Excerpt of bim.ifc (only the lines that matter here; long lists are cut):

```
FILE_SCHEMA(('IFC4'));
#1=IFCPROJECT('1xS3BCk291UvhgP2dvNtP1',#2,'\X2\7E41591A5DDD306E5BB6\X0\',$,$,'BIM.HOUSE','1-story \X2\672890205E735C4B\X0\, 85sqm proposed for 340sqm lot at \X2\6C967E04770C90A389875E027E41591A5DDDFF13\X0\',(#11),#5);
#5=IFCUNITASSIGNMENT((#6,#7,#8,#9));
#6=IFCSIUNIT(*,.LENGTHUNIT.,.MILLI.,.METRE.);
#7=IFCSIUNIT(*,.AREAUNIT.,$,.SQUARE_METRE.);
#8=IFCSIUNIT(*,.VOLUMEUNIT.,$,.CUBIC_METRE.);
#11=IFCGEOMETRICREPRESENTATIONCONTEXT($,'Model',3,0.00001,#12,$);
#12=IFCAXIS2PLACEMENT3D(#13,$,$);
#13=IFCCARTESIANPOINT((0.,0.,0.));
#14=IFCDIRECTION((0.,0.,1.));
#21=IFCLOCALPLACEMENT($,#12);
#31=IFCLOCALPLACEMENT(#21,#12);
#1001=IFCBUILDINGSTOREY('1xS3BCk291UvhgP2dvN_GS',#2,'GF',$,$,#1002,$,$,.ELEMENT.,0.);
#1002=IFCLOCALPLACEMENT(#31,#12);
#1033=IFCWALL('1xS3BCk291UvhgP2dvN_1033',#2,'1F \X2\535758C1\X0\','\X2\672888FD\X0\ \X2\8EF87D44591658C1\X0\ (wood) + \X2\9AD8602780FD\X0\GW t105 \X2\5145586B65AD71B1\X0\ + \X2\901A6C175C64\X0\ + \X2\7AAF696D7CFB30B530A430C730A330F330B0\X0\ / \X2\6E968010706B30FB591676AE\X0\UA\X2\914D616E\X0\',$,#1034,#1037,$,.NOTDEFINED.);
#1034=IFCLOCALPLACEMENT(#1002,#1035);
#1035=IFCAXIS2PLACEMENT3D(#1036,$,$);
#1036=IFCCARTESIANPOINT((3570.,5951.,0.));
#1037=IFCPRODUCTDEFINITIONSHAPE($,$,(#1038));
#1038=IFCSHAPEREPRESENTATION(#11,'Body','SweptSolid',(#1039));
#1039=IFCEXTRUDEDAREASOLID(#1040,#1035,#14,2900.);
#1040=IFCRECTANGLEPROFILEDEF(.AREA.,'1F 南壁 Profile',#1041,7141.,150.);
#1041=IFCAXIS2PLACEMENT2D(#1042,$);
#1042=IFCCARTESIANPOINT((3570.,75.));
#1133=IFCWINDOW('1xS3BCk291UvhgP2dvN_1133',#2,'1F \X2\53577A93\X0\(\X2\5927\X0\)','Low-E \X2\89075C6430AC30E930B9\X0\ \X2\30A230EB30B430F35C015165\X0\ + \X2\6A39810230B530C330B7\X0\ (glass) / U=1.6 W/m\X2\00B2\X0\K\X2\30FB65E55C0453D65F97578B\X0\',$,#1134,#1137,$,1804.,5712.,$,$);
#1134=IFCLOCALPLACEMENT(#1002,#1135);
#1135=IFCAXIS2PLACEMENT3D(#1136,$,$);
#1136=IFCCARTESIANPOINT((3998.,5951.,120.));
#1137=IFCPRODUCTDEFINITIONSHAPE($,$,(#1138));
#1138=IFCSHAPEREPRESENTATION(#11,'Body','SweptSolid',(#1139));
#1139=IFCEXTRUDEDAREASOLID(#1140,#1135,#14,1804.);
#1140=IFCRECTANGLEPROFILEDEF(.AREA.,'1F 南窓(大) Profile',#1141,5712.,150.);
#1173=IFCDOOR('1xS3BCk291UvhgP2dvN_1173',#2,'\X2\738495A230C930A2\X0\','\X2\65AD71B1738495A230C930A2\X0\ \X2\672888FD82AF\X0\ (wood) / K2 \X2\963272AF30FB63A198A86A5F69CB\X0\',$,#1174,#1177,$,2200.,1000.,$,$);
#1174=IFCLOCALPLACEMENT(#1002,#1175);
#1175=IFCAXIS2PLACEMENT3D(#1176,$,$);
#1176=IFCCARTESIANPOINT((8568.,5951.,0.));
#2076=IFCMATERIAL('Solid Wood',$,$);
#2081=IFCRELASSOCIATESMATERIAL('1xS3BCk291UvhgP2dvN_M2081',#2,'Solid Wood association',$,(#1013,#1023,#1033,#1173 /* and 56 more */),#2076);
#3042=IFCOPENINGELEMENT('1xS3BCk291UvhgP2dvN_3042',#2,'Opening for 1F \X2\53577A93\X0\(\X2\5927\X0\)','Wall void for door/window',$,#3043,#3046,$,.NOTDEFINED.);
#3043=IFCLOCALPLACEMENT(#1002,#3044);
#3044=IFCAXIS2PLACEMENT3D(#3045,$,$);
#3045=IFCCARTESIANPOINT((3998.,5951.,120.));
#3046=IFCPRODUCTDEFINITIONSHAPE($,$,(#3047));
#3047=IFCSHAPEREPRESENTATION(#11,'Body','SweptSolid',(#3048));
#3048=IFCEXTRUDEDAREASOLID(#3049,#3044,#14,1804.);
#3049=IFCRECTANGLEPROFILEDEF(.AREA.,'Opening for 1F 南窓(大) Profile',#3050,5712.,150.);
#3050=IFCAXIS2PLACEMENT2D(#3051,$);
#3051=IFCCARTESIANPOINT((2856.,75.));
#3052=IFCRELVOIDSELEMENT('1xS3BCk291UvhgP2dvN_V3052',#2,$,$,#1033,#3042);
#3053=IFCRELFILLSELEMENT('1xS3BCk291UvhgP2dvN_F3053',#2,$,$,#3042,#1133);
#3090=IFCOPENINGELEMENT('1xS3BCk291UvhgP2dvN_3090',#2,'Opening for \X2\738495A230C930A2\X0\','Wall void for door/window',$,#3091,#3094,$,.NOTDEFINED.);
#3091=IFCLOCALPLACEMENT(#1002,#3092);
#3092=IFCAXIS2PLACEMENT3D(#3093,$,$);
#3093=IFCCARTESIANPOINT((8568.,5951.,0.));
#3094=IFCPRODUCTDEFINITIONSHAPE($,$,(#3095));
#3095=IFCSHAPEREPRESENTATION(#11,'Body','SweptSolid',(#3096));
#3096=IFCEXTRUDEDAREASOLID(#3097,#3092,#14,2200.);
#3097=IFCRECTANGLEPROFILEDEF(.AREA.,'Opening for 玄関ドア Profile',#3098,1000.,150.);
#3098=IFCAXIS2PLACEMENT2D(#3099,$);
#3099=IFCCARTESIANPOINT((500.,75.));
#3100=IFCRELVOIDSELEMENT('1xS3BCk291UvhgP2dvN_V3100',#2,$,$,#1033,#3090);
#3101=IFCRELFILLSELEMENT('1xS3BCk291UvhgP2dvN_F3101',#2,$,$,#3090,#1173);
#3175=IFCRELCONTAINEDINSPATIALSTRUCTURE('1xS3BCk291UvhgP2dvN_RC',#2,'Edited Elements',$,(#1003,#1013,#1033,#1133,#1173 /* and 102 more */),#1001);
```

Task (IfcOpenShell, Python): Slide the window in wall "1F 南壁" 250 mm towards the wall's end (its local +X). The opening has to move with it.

```python
import ifcopenshell
import ifcopenshell.api.geometry
import ifcopenshell.util.placement
import ifcopenshell.util.unit

model = ifcopenshell.open("bim.ifc")
unit_scale = ifcopenshell.util.unit.calculate_unit_scale(model)

window = model.by_id(1133)
opening = window.FillsVoids[0].RelatingOpeningElement
wall = opening.VoidsElements[0].RelatingBuildingElement

wall_matrix = ifcopenshell.util.placement.get_local_placement(wall.ObjectPlacement)
shift = wall_matrix[:3, 0] * 0.25 / unit_scale
before = ifcopenshell.util.placement.get_local_placement(window.ObjectPlacement)[:3, 3].copy()

# The window is not placed relative to its opening, so move both.
for product in (opening, window):
    matrix = ifcopenshell.util.placement.get_local_placement(product.ObjectPlacement)
    matrix[:3, 3] += shift
    ifcopenshell.api.geometry.edit_object_placement(model, product=product, matrix=matrix, is_si=False)

after = ifcopenshell.util.placement.get_local_placement(window.ObjectPlacement)[:3, 3]
print("window moved by", (after - before).round(3) + 0.0)

model.write("bim_edited.ifc")
```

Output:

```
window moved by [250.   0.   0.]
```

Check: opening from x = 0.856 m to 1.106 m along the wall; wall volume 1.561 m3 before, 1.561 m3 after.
